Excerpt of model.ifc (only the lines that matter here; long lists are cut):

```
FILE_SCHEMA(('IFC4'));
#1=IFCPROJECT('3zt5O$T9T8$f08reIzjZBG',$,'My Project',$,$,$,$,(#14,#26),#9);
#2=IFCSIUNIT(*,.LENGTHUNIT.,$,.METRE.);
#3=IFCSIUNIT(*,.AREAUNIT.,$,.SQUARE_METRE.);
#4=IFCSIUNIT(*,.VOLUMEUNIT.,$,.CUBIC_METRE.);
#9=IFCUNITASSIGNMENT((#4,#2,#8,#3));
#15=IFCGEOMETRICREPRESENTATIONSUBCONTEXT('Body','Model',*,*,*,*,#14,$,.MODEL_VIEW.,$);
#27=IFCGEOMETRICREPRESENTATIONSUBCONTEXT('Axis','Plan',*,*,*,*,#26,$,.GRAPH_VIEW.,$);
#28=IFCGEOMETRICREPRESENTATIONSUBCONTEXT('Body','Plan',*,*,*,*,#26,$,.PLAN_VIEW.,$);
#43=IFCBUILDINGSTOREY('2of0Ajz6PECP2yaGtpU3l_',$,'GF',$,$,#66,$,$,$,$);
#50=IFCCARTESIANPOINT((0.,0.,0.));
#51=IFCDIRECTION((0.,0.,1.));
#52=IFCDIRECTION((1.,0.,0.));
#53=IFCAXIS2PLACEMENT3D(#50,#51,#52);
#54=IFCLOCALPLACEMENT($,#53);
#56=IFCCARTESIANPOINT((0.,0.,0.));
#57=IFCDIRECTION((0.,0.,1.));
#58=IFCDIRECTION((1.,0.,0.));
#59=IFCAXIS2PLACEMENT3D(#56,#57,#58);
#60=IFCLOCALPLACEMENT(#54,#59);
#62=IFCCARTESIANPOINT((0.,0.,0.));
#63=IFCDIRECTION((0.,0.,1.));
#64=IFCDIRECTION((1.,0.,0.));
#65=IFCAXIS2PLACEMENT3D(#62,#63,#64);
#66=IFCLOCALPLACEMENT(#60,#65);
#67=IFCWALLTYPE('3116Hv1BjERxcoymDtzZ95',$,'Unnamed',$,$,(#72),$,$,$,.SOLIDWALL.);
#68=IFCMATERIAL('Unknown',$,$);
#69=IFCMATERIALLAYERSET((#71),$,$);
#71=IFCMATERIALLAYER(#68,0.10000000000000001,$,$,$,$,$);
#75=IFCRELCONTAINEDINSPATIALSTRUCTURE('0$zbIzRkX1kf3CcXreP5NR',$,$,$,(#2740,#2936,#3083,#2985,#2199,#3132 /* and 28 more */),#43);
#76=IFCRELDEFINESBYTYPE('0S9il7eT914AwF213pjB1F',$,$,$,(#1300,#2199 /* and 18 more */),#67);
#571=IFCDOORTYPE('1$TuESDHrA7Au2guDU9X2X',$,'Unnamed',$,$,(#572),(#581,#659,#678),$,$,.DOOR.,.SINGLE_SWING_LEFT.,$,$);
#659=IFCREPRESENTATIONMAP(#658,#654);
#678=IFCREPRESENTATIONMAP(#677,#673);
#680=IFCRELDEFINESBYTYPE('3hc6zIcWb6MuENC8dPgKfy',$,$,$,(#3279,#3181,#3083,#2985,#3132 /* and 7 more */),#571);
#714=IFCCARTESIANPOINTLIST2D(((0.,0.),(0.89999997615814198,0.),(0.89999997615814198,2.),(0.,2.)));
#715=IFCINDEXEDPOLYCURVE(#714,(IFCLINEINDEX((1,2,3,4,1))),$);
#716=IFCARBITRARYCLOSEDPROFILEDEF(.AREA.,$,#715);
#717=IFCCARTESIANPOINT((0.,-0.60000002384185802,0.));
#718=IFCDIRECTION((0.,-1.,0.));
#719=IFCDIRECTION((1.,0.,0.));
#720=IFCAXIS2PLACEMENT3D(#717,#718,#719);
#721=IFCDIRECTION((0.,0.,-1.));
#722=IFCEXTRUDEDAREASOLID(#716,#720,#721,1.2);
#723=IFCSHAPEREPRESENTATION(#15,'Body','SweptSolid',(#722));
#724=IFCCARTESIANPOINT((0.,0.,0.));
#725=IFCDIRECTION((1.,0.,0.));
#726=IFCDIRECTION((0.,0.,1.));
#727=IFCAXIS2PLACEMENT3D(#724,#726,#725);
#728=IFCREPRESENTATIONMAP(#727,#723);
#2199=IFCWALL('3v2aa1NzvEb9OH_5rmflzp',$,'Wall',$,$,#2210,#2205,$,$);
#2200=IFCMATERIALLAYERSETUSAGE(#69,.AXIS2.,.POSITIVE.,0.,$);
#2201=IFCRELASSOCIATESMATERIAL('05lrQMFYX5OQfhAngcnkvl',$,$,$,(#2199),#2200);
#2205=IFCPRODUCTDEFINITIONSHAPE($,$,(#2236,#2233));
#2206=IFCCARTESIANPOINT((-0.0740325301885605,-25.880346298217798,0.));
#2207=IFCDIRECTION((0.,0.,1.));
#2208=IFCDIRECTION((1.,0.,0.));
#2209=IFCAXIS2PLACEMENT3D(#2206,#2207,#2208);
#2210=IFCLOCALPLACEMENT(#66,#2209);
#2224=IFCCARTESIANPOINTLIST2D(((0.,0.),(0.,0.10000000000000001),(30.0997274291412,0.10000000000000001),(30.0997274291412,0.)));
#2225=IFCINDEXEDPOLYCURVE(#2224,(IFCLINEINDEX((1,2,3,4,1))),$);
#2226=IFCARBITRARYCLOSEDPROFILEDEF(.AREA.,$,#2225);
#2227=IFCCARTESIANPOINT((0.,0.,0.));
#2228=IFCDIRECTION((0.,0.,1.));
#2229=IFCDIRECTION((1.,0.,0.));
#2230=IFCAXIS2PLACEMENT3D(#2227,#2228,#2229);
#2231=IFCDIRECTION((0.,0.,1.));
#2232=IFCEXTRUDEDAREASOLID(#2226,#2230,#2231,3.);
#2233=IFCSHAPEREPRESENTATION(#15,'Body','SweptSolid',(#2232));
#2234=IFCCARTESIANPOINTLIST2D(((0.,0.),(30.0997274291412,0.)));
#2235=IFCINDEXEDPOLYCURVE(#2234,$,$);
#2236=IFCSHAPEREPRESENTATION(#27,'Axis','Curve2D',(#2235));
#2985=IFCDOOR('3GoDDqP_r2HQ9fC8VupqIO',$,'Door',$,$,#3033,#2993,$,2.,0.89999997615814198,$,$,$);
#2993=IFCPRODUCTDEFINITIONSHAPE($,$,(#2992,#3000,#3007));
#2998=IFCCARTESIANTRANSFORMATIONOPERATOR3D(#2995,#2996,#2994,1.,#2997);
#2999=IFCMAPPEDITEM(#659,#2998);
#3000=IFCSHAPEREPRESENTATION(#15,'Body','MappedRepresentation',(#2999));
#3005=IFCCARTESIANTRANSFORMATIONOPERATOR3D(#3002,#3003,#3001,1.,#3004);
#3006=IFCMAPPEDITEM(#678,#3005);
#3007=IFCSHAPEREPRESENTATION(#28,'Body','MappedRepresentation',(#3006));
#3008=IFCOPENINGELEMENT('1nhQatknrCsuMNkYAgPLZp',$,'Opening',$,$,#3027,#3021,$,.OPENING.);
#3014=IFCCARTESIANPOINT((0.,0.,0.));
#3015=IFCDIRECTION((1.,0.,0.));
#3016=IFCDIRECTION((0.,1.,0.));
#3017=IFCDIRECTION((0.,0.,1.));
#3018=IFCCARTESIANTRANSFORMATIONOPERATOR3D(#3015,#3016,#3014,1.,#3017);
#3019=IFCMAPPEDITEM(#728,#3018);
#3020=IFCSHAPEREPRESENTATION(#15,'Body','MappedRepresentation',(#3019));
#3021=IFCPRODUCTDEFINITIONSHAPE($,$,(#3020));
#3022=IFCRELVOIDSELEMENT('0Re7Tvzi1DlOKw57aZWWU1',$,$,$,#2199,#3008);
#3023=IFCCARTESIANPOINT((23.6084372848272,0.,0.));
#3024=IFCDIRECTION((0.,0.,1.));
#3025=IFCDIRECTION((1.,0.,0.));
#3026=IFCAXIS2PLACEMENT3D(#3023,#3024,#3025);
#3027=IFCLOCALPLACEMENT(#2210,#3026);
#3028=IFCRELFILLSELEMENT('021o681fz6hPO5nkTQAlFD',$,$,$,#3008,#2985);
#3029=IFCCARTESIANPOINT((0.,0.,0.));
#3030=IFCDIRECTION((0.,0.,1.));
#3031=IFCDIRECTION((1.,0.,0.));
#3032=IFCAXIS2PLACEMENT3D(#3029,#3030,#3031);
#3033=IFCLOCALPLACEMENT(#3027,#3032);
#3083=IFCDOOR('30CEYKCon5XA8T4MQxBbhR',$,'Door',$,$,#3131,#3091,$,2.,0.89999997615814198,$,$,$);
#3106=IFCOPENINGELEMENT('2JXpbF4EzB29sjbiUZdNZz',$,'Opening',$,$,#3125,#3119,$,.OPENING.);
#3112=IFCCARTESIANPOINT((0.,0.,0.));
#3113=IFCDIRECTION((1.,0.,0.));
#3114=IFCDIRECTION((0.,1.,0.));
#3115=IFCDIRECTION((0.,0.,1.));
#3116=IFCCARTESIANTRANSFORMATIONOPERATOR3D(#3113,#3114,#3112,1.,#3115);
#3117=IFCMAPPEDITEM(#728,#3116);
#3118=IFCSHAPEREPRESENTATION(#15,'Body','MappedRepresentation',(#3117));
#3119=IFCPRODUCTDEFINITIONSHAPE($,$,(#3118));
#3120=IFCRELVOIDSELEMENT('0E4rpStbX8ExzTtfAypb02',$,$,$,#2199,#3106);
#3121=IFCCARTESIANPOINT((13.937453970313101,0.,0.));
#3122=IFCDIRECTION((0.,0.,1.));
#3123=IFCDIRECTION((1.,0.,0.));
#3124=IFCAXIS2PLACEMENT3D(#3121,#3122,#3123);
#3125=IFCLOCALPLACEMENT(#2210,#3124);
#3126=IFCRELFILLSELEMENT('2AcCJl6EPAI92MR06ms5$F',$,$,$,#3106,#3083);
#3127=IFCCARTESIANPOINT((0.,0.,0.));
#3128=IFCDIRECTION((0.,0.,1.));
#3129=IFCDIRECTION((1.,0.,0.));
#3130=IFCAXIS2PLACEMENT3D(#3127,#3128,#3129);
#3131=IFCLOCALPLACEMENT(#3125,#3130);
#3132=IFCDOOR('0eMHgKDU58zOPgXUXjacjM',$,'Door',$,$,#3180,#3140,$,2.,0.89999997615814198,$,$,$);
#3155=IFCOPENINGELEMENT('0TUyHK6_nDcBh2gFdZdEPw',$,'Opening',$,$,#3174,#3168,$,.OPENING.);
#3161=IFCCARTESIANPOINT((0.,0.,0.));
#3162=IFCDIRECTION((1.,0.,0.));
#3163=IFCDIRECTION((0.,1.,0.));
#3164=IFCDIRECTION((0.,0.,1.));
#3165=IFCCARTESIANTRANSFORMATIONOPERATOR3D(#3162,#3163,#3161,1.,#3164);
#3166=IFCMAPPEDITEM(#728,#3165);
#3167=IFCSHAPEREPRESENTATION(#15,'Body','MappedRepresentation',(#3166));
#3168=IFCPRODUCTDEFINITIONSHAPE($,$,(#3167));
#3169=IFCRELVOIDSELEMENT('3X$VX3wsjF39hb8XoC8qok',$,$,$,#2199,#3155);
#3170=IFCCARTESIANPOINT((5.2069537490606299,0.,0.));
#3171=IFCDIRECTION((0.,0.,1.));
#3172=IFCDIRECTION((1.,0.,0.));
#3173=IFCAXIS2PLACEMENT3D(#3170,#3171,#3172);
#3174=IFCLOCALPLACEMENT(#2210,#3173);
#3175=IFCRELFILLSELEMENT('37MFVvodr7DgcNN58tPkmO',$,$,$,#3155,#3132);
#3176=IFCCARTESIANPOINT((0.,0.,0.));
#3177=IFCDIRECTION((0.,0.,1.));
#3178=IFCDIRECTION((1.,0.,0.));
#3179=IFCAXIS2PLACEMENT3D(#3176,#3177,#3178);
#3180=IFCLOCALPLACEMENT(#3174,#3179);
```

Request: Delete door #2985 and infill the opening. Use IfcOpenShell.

```python
import ifcopenshell
import ifcopenshell.api.feature
import ifcopenshell.api.root
import ifcopenshell.geom
import ifcopenshell.util.shape

model = ifcopenshell.open("model.ifc")
settings = ifcopenshell.geom.settings()


def volume(element):
    """Net volume in cubic metres, openings subtracted."""
    shape = ifcopenshell.geom.create_shape(settings, element)
    return ifcopenshell.util.shape.get_volume(shape.geometry)


door = model.by_guid("3GoDDqP_r2HQ9fC8VupqIO")
opening = door.FillsVoids[0].RelatingOpeningElement
wall = opening.VoidsElements[0].RelatingBuildingElement
before = volume(wall)

ifcopenshell.api.root.remove_product(model, product=door)
ifcopenshell.api.feature.remove_feature(model, feature=opening)

after = volume(wall)

print(f"wall volume {before:.3f} -> {after:.3f} m3")

model.write("model-out.ifc")
```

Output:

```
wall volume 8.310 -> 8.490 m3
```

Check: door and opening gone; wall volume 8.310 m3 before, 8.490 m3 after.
